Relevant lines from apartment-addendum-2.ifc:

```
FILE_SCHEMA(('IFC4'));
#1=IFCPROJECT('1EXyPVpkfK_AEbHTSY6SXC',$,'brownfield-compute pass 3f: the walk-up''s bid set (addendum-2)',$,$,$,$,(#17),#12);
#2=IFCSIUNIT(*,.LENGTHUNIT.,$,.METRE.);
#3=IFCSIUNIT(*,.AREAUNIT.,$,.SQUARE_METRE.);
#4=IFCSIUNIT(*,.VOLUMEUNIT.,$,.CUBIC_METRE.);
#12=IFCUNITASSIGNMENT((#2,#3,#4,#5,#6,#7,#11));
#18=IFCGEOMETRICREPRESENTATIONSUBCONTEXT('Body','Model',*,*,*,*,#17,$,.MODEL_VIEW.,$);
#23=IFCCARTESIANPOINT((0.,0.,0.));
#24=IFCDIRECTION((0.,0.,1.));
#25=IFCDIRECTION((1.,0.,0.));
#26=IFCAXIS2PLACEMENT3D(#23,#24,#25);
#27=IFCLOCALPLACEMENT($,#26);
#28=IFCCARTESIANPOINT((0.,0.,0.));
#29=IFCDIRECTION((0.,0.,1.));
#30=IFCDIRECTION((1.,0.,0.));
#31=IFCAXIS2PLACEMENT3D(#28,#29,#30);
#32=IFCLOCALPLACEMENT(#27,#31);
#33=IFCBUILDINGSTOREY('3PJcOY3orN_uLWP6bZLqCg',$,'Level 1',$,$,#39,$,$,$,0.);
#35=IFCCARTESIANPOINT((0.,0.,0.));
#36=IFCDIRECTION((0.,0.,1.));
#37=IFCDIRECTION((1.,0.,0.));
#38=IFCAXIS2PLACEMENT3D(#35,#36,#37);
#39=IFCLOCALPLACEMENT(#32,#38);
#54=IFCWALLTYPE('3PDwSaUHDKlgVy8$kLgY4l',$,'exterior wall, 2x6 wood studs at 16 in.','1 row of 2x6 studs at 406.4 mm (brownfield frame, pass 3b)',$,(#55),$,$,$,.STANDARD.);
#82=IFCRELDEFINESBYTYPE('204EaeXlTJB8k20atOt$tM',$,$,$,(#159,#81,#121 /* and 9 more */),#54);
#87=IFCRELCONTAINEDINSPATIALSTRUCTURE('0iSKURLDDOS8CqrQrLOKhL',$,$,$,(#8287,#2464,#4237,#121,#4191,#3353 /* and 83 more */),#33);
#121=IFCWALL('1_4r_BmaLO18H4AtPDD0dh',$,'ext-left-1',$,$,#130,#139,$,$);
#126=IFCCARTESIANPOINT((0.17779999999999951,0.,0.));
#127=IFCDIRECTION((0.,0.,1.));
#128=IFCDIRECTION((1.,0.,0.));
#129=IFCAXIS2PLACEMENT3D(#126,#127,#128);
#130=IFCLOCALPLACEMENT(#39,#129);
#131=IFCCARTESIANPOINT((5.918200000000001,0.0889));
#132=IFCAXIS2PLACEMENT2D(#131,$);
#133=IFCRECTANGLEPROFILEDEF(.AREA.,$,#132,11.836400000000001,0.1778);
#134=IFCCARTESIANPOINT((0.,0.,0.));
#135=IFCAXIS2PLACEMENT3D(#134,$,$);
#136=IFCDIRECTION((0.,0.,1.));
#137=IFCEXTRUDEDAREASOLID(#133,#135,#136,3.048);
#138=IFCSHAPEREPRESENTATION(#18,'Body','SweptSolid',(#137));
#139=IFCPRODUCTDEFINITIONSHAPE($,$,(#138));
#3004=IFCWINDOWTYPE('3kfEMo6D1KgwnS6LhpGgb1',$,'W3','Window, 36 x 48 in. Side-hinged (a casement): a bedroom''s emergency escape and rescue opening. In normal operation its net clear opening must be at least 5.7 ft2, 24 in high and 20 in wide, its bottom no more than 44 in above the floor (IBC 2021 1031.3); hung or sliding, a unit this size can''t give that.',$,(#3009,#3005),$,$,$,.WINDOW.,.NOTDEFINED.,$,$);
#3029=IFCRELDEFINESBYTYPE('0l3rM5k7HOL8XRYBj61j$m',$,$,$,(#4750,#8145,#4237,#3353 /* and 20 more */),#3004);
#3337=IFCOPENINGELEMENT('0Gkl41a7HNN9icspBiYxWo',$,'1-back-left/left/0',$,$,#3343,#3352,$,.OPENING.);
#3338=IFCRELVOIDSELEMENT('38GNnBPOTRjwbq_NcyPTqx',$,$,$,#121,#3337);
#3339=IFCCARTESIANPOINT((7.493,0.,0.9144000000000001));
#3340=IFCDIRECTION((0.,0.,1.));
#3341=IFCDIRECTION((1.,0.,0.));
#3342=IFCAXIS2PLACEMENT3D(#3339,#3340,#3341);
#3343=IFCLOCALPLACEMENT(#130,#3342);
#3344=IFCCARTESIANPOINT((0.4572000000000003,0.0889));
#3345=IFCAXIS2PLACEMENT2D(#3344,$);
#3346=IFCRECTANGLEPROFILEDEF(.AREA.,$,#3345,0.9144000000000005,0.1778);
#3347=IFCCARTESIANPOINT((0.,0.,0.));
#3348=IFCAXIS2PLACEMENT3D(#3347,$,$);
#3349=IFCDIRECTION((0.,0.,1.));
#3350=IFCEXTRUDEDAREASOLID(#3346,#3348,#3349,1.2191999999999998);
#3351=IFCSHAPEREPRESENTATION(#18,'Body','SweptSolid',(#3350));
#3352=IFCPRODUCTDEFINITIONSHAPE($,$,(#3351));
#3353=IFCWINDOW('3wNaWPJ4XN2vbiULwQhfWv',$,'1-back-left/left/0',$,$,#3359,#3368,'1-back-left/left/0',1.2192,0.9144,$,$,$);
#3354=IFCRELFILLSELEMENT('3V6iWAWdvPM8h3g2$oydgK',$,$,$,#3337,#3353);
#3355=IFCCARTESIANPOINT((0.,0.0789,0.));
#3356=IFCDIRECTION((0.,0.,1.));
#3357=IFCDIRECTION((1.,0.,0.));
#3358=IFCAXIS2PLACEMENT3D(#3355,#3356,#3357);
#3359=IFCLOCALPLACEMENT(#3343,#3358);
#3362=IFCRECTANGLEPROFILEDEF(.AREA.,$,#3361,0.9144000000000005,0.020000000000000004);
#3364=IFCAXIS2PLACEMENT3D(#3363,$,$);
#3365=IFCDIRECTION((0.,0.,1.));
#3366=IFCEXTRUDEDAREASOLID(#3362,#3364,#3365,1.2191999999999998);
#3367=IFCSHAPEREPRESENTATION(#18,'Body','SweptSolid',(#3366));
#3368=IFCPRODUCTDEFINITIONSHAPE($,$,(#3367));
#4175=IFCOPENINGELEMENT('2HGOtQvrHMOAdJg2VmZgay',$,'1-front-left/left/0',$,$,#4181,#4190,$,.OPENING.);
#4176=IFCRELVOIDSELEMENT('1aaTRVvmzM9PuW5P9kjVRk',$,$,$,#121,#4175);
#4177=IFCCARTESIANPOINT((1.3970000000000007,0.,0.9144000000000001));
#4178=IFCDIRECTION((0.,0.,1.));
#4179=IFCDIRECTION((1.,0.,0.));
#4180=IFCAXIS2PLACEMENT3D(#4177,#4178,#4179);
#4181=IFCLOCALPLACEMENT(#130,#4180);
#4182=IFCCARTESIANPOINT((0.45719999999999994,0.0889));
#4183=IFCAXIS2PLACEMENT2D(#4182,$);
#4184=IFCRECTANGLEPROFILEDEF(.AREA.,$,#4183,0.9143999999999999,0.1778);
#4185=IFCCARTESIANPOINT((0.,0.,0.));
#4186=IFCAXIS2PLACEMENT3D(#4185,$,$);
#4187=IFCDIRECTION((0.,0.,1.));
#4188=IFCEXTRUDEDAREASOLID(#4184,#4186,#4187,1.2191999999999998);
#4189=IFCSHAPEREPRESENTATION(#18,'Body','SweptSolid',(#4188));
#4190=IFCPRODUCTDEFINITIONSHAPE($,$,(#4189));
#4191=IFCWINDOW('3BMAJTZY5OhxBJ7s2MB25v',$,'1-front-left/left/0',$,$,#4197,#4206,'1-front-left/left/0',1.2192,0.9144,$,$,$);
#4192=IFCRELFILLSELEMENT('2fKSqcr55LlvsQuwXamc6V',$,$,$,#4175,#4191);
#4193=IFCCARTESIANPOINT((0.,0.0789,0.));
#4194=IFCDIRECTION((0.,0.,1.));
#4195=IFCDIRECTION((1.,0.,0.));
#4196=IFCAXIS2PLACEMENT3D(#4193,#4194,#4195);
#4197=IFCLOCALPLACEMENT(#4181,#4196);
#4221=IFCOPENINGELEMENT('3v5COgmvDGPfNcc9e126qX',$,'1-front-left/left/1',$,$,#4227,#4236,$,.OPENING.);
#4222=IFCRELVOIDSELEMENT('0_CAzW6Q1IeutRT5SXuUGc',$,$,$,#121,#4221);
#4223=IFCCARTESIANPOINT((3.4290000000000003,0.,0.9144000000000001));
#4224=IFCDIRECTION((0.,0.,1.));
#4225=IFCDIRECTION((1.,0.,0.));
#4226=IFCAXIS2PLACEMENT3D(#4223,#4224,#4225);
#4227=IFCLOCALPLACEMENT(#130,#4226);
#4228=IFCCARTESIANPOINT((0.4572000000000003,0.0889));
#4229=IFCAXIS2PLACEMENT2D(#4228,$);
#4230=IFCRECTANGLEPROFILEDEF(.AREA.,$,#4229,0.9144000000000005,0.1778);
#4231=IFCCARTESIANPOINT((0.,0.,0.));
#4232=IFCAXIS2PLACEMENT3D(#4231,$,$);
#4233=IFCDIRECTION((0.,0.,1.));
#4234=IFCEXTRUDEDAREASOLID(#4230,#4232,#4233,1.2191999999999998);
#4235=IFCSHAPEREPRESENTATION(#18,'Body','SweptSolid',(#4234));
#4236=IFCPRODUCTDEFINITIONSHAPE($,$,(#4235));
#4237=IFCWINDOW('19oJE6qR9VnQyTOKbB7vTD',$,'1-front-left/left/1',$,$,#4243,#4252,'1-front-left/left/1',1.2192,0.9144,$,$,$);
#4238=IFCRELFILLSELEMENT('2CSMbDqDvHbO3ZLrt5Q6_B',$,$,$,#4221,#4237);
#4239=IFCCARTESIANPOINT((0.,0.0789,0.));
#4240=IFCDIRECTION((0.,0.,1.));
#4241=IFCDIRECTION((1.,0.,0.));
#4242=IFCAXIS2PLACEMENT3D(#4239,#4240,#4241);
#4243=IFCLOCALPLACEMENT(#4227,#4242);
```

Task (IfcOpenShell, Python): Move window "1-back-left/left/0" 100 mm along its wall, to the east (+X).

```python
import ifcopenshell
import ifcopenshell.api.geometry
import ifcopenshell.util.placement
import ifcopenshell.util.unit

model = ifcopenshell.open("apartment-addendum-2.ifc")
unit_scale = ifcopenshell.util.unit.calculate_unit_scale(model)

window = model.by_guid("3wNaWPJ4XN2vbiULwQhfWv")
opening = window.FillsVoids[0].RelatingOpeningElement
wall = opening.VoidsElements[0].RelatingBuildingElement

wall_matrix = ifcopenshell.util.placement.get_local_placement(wall.ObjectPlacement)
shift = wall_matrix[:3, 0] * 0.1 / unit_scale
before = ifcopenshell.util.placement.get_local_placement(window.ObjectPlacement)[:3, 3].copy()

# The window is placed relative to its opening, so it follows when the opening moves.
matrix = ifcopenshell.util.placement.get_local_placement(opening.ObjectPlacement)
matrix[:3, 3] += shift
ifcopenshell.api.geometry.edit_object_placement(
    model, product=opening, matrix=matrix, is_si=False, should_transform_children=True
)

after = ifcopenshell.util.placement.get_local_placement(window.ObjectPlacement)[:3, 3]
print("window moved by", (after - before).round(3) + 0.0)

model.write("apartment-addendum-2-out.ifc")
```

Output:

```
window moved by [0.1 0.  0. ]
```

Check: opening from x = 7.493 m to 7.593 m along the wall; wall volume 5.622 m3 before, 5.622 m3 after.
